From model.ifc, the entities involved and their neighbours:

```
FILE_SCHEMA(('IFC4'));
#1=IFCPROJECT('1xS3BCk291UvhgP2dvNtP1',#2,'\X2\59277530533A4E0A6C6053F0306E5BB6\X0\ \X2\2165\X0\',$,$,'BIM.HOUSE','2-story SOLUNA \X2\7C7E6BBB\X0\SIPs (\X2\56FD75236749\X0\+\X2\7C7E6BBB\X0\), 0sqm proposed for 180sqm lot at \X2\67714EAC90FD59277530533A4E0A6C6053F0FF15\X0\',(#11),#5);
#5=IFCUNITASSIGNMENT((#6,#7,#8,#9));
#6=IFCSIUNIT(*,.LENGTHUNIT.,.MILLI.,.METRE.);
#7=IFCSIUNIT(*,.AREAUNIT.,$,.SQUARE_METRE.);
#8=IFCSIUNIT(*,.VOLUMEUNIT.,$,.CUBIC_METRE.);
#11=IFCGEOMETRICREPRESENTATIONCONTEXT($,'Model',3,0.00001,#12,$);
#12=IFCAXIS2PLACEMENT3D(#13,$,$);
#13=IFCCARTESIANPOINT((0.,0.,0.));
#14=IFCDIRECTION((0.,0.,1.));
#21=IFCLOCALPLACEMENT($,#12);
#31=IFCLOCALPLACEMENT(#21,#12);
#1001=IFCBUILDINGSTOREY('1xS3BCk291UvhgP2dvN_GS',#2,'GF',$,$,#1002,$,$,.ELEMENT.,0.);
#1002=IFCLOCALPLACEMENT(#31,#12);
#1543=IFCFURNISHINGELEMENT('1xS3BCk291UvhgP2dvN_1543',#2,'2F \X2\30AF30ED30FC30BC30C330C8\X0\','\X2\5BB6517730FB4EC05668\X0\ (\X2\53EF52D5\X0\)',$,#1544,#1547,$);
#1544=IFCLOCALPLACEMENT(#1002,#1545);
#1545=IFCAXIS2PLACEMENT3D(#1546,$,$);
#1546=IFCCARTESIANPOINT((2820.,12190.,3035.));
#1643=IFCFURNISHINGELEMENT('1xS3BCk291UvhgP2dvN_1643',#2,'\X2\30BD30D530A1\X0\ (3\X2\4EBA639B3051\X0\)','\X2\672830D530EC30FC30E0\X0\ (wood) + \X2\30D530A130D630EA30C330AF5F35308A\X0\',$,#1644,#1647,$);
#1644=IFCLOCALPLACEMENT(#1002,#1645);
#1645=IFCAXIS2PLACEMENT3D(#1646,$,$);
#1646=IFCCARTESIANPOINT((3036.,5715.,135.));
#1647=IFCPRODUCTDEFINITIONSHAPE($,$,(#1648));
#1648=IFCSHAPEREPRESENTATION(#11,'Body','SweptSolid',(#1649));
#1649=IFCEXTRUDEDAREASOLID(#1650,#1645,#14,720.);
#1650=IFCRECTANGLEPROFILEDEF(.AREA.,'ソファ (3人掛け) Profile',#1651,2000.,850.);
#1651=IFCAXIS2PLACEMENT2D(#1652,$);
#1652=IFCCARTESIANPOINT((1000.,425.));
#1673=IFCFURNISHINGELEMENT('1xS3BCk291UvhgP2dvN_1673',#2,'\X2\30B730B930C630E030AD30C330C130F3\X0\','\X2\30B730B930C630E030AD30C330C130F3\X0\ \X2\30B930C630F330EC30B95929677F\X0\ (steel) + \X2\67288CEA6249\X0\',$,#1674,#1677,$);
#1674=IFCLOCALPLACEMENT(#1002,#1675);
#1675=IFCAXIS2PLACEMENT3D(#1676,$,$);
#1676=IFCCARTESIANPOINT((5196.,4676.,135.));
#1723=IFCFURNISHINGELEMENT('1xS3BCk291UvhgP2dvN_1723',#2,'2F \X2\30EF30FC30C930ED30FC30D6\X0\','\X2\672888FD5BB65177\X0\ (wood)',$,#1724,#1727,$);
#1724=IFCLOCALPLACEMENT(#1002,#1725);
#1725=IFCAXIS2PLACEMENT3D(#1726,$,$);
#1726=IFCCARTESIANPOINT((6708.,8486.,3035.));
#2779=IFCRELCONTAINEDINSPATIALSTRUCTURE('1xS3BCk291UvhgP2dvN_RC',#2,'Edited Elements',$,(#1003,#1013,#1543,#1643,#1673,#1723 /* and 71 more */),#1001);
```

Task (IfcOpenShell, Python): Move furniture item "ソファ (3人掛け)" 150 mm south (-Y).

```python
import ifcopenshell
import ifcopenshell.api.geometry
import ifcopenshell.util.placement

model = ifcopenshell.open("model.ifc")

item = model.by_guid("1xS3BCk291UvhgP2dvN_1643")
matrix = ifcopenshell.util.placement.get_local_placement(item.ObjectPlacement)
matrix[1, 3] -= 150.0
ifcopenshell.api.geometry.edit_object_placement(model, product=item, matrix=matrix, is_si=False)

print(ifcopenshell.util.placement.get_local_placement(item.ObjectPlacement).round(3) + 0.0)

model.write("model_v2.ifc")
```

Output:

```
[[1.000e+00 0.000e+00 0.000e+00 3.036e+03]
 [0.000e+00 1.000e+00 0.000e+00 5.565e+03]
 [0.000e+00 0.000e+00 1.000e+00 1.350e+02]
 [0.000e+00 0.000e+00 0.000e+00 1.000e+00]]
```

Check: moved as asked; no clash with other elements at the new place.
